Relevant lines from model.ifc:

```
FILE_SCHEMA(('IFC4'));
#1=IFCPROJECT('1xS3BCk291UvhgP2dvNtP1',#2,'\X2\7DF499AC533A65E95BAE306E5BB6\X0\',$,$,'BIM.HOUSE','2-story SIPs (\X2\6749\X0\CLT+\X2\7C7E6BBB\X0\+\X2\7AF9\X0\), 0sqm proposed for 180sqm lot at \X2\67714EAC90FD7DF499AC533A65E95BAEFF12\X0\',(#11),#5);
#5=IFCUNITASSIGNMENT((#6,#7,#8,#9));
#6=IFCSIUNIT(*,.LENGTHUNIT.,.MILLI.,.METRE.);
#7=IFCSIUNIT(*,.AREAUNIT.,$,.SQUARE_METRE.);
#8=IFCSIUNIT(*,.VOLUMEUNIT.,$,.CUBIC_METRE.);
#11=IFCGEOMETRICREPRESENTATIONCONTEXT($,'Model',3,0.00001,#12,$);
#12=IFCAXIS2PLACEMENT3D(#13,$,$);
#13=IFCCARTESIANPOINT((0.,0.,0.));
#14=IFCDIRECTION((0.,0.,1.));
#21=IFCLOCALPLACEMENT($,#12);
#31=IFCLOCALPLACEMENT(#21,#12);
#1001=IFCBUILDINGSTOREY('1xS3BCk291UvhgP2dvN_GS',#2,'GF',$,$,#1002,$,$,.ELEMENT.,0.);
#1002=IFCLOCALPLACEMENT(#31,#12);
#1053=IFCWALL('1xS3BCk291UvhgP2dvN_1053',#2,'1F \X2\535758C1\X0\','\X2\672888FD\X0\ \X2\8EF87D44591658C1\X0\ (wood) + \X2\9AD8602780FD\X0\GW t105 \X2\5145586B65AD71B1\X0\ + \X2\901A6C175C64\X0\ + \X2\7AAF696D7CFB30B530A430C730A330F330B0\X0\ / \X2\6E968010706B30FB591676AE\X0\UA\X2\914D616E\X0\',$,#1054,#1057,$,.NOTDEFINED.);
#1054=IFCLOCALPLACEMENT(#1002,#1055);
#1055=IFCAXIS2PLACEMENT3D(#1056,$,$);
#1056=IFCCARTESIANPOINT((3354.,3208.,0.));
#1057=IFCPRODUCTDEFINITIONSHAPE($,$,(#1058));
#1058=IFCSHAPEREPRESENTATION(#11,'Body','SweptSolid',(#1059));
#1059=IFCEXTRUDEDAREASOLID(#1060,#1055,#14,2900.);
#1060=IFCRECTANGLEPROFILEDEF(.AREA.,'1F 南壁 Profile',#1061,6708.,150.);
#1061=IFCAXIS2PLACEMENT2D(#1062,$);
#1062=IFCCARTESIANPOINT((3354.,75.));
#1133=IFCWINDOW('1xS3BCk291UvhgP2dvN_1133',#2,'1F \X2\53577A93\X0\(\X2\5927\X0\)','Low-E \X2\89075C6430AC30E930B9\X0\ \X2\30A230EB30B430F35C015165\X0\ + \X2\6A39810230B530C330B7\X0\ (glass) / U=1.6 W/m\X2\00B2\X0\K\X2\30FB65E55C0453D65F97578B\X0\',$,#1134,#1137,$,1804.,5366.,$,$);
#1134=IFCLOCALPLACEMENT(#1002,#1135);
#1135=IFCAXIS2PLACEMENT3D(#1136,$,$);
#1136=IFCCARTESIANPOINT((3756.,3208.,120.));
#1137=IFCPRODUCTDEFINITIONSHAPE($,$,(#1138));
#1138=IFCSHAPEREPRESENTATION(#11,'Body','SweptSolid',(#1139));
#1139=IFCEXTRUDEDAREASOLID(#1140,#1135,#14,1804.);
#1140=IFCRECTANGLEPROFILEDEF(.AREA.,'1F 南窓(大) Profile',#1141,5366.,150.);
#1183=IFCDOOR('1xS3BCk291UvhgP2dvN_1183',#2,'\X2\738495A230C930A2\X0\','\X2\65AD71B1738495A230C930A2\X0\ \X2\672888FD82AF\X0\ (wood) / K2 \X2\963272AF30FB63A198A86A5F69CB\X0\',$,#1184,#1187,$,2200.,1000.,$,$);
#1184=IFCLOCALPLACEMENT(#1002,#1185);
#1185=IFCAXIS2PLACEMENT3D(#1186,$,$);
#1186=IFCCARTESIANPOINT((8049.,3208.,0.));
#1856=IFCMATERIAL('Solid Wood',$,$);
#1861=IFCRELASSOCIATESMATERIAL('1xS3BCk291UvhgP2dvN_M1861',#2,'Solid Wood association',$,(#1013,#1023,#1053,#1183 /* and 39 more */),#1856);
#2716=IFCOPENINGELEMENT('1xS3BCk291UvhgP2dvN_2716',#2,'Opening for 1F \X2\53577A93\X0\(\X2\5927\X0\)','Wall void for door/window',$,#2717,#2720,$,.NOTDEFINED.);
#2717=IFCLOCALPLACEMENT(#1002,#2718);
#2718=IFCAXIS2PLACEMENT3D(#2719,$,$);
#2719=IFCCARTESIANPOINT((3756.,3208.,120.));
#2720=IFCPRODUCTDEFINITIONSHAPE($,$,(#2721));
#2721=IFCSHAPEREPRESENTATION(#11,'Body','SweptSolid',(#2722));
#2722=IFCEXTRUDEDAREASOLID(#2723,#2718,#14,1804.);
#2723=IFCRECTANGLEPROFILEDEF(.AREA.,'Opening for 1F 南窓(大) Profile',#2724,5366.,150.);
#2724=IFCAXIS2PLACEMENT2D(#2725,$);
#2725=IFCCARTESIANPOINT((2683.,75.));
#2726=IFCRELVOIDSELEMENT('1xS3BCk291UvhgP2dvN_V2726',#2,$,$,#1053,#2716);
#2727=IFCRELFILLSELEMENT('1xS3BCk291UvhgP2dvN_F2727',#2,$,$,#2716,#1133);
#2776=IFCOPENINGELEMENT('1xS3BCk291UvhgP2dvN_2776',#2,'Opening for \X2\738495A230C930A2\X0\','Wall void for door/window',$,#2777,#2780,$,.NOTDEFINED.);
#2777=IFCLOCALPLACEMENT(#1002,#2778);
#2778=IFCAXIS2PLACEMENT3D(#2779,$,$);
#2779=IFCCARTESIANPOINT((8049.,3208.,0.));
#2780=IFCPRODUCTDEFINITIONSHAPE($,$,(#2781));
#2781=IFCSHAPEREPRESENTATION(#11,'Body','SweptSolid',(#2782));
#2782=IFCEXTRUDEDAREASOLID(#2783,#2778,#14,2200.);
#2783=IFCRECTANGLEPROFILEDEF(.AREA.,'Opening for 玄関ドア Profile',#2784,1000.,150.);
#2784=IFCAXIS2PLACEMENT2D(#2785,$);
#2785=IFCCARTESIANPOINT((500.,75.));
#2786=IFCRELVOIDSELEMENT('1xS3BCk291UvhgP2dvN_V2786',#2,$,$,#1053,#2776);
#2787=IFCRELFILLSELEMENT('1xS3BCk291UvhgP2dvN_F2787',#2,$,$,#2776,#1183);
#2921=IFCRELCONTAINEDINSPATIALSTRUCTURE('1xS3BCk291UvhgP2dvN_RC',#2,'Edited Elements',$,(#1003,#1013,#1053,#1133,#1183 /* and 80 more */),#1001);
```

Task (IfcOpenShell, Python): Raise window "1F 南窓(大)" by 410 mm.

```python
import numpy as np
import ifcopenshell
import ifcopenshell.api.geometry
import ifcopenshell.util.placement
import ifcopenshell.util.unit

model = ifcopenshell.open("model.ifc")
unit_scale = ifcopenshell.util.unit.calculate_unit_scale(model)

window = model.by_guid("1xS3BCk291UvhgP2dvN_1133")
opening = window.FillsVoids[0].RelatingOpeningElement
dz = 0.41 / unit_scale

shift = np.array([0.0, 0.0, dz])
# The window is not placed relative to its opening, so move both.
for product in (opening, window):
    matrix = ifcopenshell.util.placement.get_local_placement(product.ObjectPlacement)
    matrix[:3, 3] += shift
    ifcopenshell.api.geometry.edit_object_placement(model, product=product, matrix=matrix, is_si=False)

print(f"moved by {dz * unit_scale:+.3f} m")

model.write("model-out.ifc")
```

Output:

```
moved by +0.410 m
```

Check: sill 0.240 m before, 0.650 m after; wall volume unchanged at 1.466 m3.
